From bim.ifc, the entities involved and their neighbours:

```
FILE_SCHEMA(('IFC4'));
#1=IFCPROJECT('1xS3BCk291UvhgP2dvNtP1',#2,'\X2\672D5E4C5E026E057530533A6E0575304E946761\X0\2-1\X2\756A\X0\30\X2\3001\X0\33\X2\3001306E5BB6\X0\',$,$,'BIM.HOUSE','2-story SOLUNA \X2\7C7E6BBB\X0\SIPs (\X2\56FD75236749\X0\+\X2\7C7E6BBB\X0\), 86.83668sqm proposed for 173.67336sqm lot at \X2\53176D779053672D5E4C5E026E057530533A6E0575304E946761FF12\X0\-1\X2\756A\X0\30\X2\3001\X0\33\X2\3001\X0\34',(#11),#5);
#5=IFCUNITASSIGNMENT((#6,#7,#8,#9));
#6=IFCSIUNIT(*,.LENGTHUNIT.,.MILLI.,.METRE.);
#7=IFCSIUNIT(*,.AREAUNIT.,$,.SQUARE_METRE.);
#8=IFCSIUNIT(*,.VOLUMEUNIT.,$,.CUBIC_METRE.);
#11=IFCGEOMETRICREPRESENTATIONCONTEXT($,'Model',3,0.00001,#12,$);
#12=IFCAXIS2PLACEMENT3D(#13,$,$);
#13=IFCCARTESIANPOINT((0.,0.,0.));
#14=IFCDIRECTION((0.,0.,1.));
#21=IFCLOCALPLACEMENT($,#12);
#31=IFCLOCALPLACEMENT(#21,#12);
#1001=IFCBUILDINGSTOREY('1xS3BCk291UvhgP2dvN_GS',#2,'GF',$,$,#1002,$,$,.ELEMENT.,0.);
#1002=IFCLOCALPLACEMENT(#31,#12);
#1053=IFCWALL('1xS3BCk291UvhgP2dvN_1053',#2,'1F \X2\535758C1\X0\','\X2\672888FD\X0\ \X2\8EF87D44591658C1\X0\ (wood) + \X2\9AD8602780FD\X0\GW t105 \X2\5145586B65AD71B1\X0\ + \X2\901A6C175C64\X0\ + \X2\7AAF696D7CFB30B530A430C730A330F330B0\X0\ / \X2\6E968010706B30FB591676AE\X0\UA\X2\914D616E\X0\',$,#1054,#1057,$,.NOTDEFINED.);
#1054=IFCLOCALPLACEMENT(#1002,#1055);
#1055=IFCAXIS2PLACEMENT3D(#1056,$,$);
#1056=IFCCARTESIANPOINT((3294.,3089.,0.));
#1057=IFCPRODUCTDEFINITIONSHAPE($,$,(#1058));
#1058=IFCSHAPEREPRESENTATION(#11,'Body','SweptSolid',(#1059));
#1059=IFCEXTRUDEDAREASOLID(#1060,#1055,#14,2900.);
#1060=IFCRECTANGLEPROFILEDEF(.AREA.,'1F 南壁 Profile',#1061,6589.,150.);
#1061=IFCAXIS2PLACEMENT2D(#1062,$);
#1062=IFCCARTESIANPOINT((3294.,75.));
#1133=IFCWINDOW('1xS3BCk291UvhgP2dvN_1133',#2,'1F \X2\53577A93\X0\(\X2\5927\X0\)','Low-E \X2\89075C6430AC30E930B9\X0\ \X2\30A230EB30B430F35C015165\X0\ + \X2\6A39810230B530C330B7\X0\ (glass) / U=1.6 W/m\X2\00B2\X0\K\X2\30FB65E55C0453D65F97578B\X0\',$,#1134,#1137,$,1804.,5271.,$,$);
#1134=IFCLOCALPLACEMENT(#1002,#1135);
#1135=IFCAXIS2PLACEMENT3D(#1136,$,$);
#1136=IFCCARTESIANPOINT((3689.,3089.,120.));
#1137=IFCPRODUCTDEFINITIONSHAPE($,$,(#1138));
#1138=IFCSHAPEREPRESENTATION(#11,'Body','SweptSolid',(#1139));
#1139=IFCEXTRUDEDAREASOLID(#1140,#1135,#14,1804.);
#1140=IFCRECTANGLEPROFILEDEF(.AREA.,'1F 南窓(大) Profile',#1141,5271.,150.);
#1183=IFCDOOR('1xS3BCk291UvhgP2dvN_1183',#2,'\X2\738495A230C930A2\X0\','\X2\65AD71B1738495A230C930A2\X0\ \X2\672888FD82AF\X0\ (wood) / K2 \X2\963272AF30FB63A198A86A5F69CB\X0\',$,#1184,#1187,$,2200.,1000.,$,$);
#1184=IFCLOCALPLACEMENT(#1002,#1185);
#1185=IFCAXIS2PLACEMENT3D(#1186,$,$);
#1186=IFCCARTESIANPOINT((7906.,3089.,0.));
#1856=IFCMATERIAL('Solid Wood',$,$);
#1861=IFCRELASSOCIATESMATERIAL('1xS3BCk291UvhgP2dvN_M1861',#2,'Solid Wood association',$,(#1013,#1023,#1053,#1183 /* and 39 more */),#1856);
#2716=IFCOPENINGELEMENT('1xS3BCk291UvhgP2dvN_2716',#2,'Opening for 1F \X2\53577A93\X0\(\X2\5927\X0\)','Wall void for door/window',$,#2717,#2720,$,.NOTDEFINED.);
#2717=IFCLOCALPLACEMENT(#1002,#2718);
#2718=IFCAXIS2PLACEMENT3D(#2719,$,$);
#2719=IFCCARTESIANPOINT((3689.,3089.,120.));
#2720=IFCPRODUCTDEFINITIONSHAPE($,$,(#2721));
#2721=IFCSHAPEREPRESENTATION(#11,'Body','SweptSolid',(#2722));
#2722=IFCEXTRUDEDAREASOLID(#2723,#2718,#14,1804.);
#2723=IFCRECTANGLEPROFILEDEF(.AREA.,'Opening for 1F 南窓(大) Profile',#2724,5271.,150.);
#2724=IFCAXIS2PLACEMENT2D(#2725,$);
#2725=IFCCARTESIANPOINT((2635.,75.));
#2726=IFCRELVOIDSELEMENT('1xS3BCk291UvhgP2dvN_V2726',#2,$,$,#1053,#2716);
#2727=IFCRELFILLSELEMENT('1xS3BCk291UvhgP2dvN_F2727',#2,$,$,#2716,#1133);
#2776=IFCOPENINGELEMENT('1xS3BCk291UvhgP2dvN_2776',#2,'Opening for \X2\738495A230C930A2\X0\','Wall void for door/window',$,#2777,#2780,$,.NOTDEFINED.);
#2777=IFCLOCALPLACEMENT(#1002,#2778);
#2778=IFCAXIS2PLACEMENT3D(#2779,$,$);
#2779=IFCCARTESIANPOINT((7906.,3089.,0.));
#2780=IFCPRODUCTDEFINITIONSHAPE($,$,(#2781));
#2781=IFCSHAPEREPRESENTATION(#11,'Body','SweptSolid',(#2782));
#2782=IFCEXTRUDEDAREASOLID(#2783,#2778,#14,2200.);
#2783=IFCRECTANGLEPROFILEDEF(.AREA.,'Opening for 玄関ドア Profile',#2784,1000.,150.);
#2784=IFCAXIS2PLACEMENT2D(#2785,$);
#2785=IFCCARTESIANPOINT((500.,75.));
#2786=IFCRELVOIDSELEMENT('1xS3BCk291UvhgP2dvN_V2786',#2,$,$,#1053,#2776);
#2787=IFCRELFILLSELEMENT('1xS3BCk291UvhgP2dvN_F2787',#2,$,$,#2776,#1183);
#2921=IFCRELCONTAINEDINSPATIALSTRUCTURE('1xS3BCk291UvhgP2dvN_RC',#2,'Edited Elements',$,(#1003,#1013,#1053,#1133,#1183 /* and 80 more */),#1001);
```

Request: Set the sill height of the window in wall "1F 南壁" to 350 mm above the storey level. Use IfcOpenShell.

```python
import numpy as np
import ifcopenshell
import ifcopenshell.api.geometry
import ifcopenshell.geom
import ifcopenshell.util.element
import ifcopenshell.util.placement
import ifcopenshell.util.shape
import ifcopenshell.util.unit

model = ifcopenshell.open("bim.ifc")
unit_scale = ifcopenshell.util.unit.calculate_unit_scale(model)

window = model.by_guid("1xS3BCk291UvhgP2dvN_1133")
opening = window.FillsVoids[0].RelatingOpeningElement
storey = ifcopenshell.util.element.get_container(window, ifc_class="IfcBuildingStorey")
level = ifcopenshell.util.placement.get_local_placement(storey.ObjectPlacement)[2, 3]

# The opening's origin need not be at the sill, so measure its lowest point.
shape = ifcopenshell.geom.create_shape(ifcopenshell.geom.settings(), opening)
bottom = ifcopenshell.util.shape.get_shape_bottom_elevation(shape, shape.geometry) / unit_scale
dz = level + 350.0 - bottom

shift = np.array([0.0, 0.0, dz])
# The window is not placed relative to its opening, so move both.
for product in (opening, window):
    matrix = ifcopenshell.util.placement.get_local_placement(product.ObjectPlacement)
    matrix[:3, 3] += shift
    ifcopenshell.api.geometry.edit_object_placement(model, product=product, matrix=matrix, is_si=False)

print(f"moved by {dz * unit_scale:+.3f} m")

model.write("bim-out.ifc")
```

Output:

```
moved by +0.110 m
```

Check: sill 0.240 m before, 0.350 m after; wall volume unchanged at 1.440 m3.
